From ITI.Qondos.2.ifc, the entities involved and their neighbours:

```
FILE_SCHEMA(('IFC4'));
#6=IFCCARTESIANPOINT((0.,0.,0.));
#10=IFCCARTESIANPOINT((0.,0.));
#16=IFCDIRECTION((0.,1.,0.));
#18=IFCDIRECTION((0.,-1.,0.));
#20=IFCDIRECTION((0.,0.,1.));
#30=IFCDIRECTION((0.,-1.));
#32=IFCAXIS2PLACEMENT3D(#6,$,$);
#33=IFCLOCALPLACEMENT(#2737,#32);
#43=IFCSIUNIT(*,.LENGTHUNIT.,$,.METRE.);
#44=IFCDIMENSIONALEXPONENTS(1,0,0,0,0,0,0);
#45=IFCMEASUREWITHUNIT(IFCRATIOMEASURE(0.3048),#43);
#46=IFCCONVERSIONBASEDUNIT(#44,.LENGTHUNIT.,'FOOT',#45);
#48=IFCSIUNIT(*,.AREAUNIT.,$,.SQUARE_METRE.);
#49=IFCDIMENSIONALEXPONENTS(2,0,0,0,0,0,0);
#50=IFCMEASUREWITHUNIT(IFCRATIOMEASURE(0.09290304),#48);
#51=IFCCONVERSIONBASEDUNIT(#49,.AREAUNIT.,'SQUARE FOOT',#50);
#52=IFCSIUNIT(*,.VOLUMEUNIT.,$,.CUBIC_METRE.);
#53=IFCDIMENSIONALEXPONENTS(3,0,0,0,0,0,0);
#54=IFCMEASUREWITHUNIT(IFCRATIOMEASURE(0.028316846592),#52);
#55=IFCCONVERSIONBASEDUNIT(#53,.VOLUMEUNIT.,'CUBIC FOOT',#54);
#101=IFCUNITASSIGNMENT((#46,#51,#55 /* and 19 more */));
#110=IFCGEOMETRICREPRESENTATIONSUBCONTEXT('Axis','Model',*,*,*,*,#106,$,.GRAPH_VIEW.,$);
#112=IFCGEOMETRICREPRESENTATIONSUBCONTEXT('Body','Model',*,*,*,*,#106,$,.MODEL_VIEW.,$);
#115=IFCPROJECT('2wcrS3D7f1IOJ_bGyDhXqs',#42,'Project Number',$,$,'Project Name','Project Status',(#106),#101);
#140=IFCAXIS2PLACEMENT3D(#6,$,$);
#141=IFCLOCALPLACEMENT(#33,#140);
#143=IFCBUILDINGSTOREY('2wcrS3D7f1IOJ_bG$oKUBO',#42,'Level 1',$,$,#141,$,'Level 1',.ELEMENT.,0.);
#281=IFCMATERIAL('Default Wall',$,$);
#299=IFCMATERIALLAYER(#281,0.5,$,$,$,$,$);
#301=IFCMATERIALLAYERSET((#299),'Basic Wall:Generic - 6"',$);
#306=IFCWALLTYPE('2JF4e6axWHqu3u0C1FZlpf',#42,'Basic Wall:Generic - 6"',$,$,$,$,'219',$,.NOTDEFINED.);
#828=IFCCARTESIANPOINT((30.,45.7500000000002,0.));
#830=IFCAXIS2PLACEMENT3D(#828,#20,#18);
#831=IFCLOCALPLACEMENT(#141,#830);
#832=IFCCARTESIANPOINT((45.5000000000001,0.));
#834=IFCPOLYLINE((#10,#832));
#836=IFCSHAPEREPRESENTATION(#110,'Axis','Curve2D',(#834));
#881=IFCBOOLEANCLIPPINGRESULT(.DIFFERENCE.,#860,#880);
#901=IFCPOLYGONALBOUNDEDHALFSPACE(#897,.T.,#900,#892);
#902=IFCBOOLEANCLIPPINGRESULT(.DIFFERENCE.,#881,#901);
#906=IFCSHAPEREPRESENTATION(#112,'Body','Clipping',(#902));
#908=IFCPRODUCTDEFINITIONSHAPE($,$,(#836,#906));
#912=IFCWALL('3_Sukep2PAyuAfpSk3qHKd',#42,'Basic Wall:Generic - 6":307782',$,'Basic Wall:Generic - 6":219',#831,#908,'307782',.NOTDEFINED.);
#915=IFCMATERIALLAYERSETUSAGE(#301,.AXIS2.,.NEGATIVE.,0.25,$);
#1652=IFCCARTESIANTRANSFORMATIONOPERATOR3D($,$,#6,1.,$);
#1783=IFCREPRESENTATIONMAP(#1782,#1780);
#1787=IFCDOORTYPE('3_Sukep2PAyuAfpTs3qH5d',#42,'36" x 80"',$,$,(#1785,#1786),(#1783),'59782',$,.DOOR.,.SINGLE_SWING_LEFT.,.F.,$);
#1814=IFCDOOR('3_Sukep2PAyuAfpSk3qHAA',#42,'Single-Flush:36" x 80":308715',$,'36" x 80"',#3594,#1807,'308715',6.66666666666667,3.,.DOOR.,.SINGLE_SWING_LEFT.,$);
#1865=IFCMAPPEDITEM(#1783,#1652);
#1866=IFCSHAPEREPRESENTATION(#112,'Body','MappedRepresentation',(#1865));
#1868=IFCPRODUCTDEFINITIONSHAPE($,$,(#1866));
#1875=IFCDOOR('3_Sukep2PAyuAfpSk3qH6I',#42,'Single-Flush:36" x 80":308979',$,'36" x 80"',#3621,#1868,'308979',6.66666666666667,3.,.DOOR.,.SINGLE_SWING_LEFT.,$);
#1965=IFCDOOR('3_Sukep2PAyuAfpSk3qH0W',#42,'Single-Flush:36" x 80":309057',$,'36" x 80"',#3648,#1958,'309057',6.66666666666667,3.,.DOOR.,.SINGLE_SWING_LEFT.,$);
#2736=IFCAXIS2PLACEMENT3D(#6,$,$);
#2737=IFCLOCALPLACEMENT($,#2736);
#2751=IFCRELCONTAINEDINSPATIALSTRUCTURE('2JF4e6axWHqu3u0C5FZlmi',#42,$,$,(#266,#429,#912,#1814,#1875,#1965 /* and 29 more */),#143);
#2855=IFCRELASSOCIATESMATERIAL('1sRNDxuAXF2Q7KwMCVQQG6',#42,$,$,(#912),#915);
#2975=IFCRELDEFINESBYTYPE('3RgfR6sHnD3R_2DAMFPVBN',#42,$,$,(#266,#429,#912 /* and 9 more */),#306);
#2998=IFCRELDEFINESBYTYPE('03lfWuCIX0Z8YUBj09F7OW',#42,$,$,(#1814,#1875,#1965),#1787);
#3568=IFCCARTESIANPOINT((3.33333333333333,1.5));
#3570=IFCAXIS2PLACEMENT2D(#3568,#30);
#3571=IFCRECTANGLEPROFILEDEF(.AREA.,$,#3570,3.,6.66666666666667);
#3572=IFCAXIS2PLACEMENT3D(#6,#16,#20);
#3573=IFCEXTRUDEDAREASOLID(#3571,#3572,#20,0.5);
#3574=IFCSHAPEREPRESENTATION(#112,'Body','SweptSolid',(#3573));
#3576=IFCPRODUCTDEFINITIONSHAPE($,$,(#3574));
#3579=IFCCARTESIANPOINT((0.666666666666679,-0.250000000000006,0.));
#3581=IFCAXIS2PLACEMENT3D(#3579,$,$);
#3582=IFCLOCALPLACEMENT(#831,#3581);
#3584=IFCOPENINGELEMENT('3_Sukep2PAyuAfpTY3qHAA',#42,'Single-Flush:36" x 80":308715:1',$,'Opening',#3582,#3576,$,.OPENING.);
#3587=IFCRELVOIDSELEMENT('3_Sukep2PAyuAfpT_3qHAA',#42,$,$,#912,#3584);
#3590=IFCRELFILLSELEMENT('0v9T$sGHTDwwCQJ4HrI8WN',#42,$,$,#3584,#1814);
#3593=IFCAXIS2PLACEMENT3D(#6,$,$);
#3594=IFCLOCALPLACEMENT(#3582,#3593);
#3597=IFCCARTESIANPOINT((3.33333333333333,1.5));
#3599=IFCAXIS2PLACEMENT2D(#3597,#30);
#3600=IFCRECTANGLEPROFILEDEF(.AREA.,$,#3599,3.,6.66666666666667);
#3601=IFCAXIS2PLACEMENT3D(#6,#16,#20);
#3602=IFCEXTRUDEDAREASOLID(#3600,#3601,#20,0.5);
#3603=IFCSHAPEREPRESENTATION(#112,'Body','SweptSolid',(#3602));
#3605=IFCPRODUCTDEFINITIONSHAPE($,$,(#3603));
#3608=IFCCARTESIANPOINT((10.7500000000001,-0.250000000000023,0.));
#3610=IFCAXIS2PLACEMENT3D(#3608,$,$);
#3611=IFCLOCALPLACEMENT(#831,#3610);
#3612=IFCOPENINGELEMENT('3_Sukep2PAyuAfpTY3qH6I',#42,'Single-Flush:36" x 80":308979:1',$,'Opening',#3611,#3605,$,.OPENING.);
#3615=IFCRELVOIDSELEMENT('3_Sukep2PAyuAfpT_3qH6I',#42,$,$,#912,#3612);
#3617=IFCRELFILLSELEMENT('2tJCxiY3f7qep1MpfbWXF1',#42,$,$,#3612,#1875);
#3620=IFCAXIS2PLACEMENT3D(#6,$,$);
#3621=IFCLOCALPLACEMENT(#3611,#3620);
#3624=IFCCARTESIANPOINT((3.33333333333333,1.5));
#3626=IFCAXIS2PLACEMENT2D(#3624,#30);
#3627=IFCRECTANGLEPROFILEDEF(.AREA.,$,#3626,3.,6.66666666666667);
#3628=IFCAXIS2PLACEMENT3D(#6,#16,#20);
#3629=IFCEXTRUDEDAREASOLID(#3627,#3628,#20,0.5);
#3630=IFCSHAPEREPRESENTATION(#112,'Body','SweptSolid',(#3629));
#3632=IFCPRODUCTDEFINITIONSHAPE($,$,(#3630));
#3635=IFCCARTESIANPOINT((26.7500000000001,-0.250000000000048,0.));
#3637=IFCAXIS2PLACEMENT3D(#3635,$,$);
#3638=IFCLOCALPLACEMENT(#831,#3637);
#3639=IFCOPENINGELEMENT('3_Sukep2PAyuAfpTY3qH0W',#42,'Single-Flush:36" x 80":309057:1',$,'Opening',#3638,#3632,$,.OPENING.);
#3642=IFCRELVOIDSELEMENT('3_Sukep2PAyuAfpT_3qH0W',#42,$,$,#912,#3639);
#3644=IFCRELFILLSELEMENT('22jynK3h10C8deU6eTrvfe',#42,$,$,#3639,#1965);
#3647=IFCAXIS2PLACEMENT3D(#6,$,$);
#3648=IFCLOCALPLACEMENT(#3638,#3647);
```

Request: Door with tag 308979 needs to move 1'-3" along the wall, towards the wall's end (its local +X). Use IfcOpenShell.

```python
import ifcopenshell
import ifcopenshell.api.geometry
import ifcopenshell.util.placement
import ifcopenshell.util.unit

model = ifcopenshell.open("ITI.Qondos.2.ifc")
unit_scale = ifcopenshell.util.unit.calculate_unit_scale(model)

door = model.by_id(1875)
opening = door.FillsVoids[0].RelatingOpeningElement
wall = opening.VoidsElements[0].RelatingBuildingElement

wall_matrix = ifcopenshell.util.placement.get_local_placement(wall.ObjectPlacement)
shift = wall_matrix[:3, 0] * 15 * 0.0254 / unit_scale
before = ifcopenshell.util.placement.get_local_placement(door.ObjectPlacement)[:3, 3].copy()

# The door is placed relative to its opening, so it follows when the opening moves.
matrix = ifcopenshell.util.placement.get_local_placement(opening.ObjectPlacement)
matrix[:3, 3] += shift
ifcopenshell.api.geometry.edit_object_placement(
    model, product=opening, matrix=matrix, is_si=False, should_transform_children=True
)

after = ifcopenshell.util.placement.get_local_placement(door.ObjectPlacement)[:3, 3]
print("door moved by", (after - before).round(3) + 0.0)

model.write("ITI.Qondos.2_edited.ifc")
```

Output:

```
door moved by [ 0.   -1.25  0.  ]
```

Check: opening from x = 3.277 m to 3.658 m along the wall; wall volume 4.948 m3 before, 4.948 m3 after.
